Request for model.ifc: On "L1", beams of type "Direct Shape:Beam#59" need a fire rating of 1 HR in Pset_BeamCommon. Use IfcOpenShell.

First a look at what the model holds.

```python
import ifcopenshell
import ifcopenshell.util.element

model = ifcopenshell.open("model.ifc")
print(model.schema)
storey = next(s for s in model.by_type("IfcBuildingStorey") if s.Name == "L1")
beams = [e for e in ifcopenshell.util.element.get_decomposition(storey) if e.is_a("IfcBeam")]
seen = {}
for e in beams:
    element_type = ifcopenshell.util.element.get_type(e)
    key = (element_type.Name if element_type != e and element_type else None, ifcopenshell.util.element.get_pset(e, "Pset_BeamCommon", "FireRating"))
    seen[key] = seen.get(key, 0) + 1
for (name, value), count in sorted(seen.items(), key=str):
    print(count, "x", name, "|", value)
```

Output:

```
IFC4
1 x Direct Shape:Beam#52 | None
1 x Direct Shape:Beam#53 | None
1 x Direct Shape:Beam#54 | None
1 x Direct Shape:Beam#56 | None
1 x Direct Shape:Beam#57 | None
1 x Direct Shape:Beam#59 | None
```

```python
import ifcopenshell
import ifcopenshell.api.pset
import ifcopenshell.util.element

model = ifcopenshell.open("model.ifc")

storey = next(s for s in model.by_type("IfcBuildingStorey") if s.Name == "L1")
beams = [e for e in ifcopenshell.util.element.get_decomposition(storey) if e.is_a("IfcBeam")]

count = 0
for e in beams:
    element_type = ifcopenshell.util.element.get_type(e)
    if element_type in (None, e) or element_type.Name != "Direct Shape:Beam#59":
        continue
    # add_pset returns the element's existing set when there is one.
    pset = ifcopenshell.api.pset.add_pset(model, product=e, name="Pset_BeamCommon")
    ifcopenshell.api.pset.edit_pset(model, pset=pset, properties={"FireRating": "1 HR"})
    count += 1

print(count, "beams updated")

model.write("model_edited.ifc")
```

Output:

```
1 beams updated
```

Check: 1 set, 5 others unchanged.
